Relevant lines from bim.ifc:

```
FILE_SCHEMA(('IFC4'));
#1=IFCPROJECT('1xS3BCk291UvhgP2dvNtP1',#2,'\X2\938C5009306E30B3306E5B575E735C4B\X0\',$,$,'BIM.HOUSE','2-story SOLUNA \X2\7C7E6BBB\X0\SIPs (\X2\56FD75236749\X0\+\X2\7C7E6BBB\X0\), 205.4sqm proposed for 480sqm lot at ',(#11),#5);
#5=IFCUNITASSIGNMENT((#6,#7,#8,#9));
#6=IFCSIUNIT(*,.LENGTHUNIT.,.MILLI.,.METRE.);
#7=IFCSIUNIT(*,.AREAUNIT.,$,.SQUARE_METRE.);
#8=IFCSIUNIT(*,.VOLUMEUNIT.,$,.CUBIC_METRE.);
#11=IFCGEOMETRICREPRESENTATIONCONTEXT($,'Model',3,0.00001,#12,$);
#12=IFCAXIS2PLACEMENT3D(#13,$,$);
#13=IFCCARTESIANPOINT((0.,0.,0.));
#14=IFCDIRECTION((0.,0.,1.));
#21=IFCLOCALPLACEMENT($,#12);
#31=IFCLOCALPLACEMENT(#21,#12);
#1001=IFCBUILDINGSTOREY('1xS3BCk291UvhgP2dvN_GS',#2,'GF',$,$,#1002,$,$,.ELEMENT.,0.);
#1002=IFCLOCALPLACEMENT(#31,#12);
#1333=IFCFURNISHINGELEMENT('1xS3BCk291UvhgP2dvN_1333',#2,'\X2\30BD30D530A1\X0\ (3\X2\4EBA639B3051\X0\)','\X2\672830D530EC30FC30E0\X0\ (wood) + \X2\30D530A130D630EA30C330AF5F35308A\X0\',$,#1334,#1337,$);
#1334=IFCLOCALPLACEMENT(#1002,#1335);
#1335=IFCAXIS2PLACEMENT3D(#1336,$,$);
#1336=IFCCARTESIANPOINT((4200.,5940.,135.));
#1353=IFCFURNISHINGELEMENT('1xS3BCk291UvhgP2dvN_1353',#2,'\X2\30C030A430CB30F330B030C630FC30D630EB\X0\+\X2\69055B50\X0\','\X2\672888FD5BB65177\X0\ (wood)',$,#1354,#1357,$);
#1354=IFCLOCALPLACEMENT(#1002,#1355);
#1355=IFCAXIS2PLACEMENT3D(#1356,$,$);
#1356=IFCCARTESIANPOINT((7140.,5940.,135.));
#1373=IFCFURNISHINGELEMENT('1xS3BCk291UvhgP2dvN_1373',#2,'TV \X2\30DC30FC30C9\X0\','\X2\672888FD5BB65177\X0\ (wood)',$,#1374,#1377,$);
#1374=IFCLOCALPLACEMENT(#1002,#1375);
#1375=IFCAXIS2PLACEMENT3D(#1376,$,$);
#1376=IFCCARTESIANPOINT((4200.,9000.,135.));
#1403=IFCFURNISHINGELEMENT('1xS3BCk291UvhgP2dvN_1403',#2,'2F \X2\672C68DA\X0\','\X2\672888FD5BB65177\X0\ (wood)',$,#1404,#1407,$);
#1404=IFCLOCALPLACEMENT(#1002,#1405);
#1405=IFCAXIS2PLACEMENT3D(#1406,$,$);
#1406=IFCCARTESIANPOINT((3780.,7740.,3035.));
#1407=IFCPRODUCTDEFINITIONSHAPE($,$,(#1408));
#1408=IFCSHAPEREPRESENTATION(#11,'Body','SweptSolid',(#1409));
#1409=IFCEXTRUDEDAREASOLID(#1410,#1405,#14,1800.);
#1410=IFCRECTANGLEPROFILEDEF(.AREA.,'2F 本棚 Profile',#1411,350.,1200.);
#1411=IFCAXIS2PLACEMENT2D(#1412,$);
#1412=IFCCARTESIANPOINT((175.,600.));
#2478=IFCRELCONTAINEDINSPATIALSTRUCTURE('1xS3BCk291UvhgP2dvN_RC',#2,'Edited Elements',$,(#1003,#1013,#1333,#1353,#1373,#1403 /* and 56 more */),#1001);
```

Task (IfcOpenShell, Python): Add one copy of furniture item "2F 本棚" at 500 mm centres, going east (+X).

```python
import numpy as np
import ifcopenshell
import ifcopenshell.api.geometry
import ifcopenshell.api.root
import ifcopenshell.util.element
import ifcopenshell.util.placement
import ifcopenshell.util.unit

model = ifcopenshell.open("bim.ifc")
unit_scale = ifcopenshell.util.unit.calculate_unit_scale(model)


def reuse_history(source, copy):
    """copy_class also copies each property set's owner history, people and application; keep the originals."""
    for rel in copy.IsDefinedBy:
        if rel.is_a("IfcRelDefinesByProperties") and (history := rel.RelatingPropertyDefinition.OwnerHistory):
            rel.RelatingPropertyDefinition.OwnerHistory = source.OwnerHistory
            ifcopenshell.util.element.remove_deep2(model, history)


source = model.by_guid("1xS3BCk291UvhgP2dvN_1403")
base = ifcopenshell.util.placement.get_local_placement(source.ObjectPlacement)
step = np.array([1.0, 0.0, 0.0]) * 0.5 / unit_scale

for i in range(1, 2):
    copy = ifcopenshell.api.root.copy_class(model, product=source)
    copy.Representation = ifcopenshell.util.element.copy_deep(
        model, source.Representation, exclude=["IfcGeometricRepresentationContext", "IfcRepresentationMap"]
    )
    reuse_history(source, copy)
    matrix = base.copy()
    matrix[:3, 3] += i * step
    print("added at", matrix[:3, 3].round(3) + 0.0)
    ifcopenshell.api.geometry.edit_object_placement(model, product=copy, matrix=matrix, is_si=False)

model.write("bim-out.ifc")
```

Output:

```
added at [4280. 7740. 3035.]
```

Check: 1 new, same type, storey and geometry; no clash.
